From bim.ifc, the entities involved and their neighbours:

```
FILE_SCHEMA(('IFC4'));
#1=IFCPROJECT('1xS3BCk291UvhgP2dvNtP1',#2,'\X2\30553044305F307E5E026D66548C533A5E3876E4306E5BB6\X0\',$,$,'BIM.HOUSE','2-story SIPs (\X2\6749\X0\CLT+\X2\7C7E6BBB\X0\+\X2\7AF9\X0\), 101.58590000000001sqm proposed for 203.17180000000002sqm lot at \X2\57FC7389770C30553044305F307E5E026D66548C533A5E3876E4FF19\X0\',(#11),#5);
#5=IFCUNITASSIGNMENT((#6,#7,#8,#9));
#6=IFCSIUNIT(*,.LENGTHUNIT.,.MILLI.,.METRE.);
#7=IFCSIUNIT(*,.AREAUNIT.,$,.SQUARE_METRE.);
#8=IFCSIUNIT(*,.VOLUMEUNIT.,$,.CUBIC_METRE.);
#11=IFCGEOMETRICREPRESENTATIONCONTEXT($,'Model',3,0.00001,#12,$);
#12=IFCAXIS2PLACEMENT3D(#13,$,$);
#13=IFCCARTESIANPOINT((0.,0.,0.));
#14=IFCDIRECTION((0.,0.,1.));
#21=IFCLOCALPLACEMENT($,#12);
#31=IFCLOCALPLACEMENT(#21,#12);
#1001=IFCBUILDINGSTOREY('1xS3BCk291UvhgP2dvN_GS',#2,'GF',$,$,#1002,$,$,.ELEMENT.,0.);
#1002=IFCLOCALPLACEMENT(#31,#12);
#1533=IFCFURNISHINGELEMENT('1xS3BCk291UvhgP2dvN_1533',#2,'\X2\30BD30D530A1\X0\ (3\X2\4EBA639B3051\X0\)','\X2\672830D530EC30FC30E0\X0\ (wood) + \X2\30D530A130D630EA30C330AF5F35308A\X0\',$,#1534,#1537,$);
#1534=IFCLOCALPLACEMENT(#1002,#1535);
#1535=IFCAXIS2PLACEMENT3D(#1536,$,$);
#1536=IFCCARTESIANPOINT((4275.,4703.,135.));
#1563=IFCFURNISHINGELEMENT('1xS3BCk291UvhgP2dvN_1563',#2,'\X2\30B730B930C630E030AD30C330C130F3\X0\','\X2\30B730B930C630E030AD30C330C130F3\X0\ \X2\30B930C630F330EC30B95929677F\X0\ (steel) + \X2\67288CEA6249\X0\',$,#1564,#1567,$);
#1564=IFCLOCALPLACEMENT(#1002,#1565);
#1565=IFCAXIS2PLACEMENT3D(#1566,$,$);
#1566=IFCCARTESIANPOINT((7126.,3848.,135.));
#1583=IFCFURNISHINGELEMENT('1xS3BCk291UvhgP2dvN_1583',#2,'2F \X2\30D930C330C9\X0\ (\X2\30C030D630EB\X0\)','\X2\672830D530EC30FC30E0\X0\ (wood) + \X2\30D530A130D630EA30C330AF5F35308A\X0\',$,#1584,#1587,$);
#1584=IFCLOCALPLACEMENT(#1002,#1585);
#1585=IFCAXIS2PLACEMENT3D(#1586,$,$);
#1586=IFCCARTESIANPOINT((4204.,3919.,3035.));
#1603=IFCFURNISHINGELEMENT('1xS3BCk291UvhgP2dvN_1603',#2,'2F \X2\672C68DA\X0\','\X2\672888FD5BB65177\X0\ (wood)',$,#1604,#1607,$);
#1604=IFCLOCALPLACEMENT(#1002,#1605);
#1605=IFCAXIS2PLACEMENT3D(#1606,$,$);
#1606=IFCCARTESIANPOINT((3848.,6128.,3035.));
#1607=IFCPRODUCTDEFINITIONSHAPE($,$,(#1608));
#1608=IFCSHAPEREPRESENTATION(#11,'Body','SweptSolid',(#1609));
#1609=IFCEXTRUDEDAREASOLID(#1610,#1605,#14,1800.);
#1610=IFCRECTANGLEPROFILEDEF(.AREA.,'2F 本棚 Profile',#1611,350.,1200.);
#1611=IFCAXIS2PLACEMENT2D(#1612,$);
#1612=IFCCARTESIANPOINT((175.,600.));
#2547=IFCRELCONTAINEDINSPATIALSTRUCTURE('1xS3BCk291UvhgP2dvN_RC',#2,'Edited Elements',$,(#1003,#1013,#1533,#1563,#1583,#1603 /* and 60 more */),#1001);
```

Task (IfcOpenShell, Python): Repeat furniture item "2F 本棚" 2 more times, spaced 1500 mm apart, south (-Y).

```python
import numpy as np
import ifcopenshell
import ifcopenshell.api.geometry
import ifcopenshell.api.root
import ifcopenshell.util.element
import ifcopenshell.util.placement
import ifcopenshell.util.unit

model = ifcopenshell.open("bim.ifc")
unit_scale = ifcopenshell.util.unit.calculate_unit_scale(model)


def reuse_history(source, copy):
    """copy_class also copies each property set's owner history, people and application; keep the originals."""
    for rel in copy.IsDefinedBy:
        if rel.is_a("IfcRelDefinesByProperties") and (history := rel.RelatingPropertyDefinition.OwnerHistory):
            rel.RelatingPropertyDefinition.OwnerHistory = source.OwnerHistory
            ifcopenshell.util.element.remove_deep2(model, history)


source = model.by_id(1603)
base = ifcopenshell.util.placement.get_local_placement(source.ObjectPlacement)
step = np.array([0.0, -1.0, 0.0]) * 1.5 / unit_scale

for i in range(1, 3):
    copy = ifcopenshell.api.root.copy_class(model, product=source)
    copy.Representation = ifcopenshell.util.element.copy_deep(
        model, source.Representation, exclude=["IfcGeometricRepresentationContext", "IfcRepresentationMap"]
    )
    reuse_history(source, copy)
    matrix = base.copy()
    matrix[:3, 3] += i * step
    print("added at", matrix[:3, 3].round(3) + 0.0)
    ifcopenshell.api.geometry.edit_object_placement(model, product=copy, matrix=matrix, is_si=False)

model.write("bim_updated.ifc")
```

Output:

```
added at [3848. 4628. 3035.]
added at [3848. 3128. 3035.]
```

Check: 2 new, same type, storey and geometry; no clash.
